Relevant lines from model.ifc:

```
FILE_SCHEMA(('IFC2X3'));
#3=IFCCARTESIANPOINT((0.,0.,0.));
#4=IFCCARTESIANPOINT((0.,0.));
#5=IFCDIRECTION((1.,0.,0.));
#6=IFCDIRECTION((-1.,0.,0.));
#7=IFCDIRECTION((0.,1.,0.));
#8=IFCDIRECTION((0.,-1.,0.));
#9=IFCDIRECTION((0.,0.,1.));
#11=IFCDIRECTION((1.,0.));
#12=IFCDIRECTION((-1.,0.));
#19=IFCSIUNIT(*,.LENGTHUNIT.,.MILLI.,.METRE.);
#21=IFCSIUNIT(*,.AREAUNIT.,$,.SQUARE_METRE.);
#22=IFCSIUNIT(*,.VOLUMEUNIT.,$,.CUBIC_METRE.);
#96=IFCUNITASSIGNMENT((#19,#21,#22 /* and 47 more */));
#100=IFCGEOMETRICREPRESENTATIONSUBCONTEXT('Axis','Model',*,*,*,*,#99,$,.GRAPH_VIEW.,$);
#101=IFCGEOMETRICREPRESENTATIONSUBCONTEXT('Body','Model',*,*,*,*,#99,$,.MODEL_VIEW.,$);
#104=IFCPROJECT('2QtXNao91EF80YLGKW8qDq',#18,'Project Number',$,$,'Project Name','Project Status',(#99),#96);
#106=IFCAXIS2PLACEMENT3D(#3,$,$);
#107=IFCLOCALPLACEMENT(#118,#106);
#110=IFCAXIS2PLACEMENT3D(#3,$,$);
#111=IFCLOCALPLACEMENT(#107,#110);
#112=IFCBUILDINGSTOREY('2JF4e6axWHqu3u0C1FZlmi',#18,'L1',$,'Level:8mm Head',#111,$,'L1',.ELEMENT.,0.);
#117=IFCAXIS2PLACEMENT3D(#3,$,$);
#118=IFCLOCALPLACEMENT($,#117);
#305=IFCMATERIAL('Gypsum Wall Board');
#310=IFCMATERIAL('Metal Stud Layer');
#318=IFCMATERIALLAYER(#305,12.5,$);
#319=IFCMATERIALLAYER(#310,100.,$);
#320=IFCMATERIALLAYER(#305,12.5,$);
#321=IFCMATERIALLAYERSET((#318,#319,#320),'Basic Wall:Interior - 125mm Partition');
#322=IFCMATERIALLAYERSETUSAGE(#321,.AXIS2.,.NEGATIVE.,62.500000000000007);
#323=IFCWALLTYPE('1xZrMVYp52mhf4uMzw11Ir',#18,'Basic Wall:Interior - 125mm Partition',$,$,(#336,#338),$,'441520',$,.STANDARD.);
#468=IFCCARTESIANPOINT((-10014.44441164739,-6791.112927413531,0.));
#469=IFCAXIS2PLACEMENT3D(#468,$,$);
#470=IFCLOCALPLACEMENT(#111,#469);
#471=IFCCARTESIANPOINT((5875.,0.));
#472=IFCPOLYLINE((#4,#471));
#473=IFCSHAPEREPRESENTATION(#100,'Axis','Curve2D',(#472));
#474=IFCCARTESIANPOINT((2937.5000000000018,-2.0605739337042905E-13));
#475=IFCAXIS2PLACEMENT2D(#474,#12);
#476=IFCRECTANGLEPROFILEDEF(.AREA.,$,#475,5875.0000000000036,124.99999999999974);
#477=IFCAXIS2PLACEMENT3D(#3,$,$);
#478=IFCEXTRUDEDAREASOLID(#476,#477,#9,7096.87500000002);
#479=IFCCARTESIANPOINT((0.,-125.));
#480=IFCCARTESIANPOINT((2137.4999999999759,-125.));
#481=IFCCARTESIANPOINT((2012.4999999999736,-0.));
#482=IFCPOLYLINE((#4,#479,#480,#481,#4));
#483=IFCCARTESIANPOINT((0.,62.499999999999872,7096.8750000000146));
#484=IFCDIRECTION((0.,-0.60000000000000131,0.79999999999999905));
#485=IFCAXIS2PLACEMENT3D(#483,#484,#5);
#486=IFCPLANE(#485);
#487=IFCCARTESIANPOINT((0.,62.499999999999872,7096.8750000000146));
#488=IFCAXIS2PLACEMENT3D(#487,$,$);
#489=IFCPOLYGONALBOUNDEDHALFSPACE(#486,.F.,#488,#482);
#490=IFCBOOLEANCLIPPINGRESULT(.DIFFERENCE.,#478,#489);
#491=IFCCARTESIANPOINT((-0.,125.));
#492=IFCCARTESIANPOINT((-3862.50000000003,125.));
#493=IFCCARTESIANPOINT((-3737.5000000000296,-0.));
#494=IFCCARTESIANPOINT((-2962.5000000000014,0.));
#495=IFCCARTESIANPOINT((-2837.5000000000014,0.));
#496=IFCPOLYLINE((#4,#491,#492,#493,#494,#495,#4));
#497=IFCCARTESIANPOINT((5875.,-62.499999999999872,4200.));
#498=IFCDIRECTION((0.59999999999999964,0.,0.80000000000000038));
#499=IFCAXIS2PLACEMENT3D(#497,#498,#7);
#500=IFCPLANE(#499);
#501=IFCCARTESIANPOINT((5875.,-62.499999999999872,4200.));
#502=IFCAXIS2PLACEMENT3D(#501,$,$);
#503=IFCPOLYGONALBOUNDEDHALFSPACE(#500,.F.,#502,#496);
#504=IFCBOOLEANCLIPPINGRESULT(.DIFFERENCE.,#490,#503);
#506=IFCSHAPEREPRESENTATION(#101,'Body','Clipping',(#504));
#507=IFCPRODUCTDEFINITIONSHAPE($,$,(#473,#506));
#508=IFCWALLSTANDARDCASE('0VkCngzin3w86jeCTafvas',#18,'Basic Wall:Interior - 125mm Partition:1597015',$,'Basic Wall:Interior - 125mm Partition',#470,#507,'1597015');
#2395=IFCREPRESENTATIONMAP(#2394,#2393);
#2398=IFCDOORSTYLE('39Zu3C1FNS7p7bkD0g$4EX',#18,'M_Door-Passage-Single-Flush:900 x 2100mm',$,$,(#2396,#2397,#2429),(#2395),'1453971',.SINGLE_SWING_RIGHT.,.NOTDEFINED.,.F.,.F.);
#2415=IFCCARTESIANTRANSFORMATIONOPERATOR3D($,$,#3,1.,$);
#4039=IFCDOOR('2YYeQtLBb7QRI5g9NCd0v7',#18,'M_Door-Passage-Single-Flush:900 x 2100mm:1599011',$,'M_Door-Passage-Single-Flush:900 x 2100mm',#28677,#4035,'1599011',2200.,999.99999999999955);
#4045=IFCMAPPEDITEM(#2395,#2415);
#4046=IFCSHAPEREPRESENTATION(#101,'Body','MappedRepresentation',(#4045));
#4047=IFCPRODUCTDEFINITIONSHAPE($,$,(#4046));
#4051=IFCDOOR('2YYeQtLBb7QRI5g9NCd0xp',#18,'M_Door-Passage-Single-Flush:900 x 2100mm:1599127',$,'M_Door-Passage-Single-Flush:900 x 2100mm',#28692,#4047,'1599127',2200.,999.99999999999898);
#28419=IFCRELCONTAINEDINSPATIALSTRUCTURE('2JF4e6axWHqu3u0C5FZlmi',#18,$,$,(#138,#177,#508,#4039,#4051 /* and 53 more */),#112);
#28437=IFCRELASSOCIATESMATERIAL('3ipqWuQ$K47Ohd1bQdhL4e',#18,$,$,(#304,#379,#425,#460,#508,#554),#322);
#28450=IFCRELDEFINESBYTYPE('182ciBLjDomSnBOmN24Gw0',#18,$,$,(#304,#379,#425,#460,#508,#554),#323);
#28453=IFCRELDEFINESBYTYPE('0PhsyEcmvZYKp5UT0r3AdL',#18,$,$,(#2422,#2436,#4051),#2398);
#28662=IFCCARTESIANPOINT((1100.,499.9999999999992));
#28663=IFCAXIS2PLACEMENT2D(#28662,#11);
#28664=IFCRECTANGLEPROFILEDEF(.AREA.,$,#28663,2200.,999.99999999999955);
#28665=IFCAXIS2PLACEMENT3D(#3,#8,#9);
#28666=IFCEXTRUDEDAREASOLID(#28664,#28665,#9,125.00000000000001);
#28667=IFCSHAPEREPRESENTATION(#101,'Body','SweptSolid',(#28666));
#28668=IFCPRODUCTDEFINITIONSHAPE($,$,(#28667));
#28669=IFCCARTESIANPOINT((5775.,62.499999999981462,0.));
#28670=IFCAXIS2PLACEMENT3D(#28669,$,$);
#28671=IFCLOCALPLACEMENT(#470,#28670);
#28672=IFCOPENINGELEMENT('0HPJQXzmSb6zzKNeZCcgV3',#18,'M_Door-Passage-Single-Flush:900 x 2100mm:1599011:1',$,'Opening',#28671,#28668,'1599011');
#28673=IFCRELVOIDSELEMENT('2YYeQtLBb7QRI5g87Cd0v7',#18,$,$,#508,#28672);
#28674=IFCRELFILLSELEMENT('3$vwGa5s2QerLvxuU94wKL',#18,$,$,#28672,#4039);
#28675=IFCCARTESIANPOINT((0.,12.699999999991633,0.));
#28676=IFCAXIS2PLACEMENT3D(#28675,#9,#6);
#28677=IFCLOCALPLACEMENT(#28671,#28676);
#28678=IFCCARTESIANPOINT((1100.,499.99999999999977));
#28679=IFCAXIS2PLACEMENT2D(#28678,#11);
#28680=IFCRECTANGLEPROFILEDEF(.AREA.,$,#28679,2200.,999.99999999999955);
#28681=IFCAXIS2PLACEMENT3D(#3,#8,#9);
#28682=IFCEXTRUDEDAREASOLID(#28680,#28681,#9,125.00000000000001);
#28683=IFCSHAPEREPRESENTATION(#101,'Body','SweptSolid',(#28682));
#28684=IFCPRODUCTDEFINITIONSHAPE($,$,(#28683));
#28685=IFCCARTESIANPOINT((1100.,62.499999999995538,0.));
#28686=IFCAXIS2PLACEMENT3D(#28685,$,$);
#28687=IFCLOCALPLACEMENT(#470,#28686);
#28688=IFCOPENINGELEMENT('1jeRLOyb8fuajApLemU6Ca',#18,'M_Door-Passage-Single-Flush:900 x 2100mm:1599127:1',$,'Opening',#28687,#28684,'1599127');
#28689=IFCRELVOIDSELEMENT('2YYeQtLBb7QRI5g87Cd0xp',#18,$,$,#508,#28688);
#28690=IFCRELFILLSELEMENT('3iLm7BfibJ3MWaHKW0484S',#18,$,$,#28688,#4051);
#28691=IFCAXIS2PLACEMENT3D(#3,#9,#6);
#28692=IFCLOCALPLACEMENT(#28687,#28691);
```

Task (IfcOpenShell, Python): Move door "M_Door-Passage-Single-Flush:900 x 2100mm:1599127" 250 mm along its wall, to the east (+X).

```python
import ifcopenshell
import ifcopenshell.api.geometry
import ifcopenshell.util.placement

model = ifcopenshell.open("model.ifc")

door = model.by_guid("2YYeQtLBb7QRI5g9NCd0xp")
opening = door.FillsVoids[0].RelatingOpeningElement
wall = opening.VoidsElements[0].RelatingBuildingElement

wall_matrix = ifcopenshell.util.placement.get_local_placement(wall.ObjectPlacement)
shift = wall_matrix[:3, 0] * 250.0
before = ifcopenshell.util.placement.get_local_placement(door.ObjectPlacement)[:3, 3].copy()

# The door is placed relative to its opening, so it follows when the opening moves.
matrix = ifcopenshell.util.placement.get_local_placement(opening.ObjectPlacement)
matrix[:3, 3] += shift
ifcopenshell.api.geometry.edit_object_placement(
    model, product=opening, matrix=matrix, is_si=False, should_transform_children=True
)

after = ifcopenshell.util.placement.get_local_placement(door.ObjectPlacement)[:3, 3]
print("door moved by", (after - before).round(3) + 0.0)

model.write("model_v2.ifc")
```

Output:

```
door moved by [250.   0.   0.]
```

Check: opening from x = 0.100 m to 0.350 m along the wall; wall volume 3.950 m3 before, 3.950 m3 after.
